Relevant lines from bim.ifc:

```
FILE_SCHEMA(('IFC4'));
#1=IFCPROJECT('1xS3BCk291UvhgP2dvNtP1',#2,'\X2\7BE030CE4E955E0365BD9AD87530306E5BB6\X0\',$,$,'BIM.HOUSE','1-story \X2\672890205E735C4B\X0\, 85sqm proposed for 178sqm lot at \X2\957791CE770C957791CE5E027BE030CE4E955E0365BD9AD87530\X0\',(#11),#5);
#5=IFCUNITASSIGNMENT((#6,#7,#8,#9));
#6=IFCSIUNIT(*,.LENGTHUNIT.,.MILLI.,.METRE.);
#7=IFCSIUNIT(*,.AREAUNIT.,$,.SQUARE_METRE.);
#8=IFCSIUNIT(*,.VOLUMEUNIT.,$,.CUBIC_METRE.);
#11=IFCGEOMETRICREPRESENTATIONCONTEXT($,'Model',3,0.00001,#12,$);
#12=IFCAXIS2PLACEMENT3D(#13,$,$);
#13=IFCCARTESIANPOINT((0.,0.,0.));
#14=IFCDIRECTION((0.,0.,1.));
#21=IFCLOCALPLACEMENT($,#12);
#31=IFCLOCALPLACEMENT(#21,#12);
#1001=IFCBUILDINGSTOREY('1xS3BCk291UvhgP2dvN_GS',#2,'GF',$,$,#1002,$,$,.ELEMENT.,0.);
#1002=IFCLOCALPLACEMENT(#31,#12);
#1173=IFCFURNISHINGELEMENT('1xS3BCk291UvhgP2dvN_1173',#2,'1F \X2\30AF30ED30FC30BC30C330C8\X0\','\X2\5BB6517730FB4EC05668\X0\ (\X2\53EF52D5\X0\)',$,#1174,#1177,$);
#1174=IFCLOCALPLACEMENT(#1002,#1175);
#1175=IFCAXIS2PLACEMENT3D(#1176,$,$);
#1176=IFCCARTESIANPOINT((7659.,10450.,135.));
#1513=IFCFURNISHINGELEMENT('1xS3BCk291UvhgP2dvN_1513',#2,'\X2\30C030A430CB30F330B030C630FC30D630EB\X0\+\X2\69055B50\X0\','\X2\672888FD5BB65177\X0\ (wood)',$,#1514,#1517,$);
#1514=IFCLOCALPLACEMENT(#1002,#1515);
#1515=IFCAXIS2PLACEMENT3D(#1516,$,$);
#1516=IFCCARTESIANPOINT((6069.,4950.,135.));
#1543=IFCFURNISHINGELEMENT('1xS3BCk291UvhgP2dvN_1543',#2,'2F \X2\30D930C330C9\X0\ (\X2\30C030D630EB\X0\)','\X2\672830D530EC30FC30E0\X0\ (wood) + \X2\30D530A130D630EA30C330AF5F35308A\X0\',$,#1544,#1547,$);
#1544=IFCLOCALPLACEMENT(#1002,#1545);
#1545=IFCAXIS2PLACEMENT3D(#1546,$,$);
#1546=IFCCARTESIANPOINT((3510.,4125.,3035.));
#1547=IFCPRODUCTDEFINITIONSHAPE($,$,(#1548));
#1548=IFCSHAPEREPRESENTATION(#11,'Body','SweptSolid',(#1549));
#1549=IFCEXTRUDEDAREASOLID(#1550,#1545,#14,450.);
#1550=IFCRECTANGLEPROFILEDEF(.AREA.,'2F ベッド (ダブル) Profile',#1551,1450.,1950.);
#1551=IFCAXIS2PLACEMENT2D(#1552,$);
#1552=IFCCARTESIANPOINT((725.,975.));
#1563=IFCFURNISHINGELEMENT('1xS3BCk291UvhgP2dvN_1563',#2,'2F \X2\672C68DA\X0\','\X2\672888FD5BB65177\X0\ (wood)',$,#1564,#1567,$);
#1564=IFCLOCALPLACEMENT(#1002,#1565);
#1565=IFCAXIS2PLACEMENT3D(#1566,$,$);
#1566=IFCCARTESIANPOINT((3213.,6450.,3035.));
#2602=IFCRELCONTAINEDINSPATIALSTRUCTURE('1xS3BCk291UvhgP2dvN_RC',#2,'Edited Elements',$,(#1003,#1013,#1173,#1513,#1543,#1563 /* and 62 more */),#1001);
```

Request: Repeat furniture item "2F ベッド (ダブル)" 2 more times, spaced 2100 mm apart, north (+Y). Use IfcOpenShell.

```python
import numpy as np
import ifcopenshell
import ifcopenshell.api.geometry
import ifcopenshell.api.root
import ifcopenshell.util.element
import ifcopenshell.util.placement
import ifcopenshell.util.unit

model = ifcopenshell.open("bim.ifc")
unit_scale = ifcopenshell.util.unit.calculate_unit_scale(model)


def reuse_history(source, copy):
    """copy_class also copies each property set's owner history, people and application; keep the originals."""
    for rel in copy.IsDefinedBy:
        if rel.is_a("IfcRelDefinesByProperties") and (history := rel.RelatingPropertyDefinition.OwnerHistory):
            rel.RelatingPropertyDefinition.OwnerHistory = source.OwnerHistory
            ifcopenshell.util.element.remove_deep2(model, history)


source = model.by_id(1543)
base = ifcopenshell.util.placement.get_local_placement(source.ObjectPlacement)
step = np.array([0.0, 1.0, 0.0]) * 2.1 / unit_scale

for i in range(1, 3):
    copy = ifcopenshell.api.root.copy_class(model, product=source)
    copy.Representation = ifcopenshell.util.element.copy_deep(
        model, source.Representation, exclude=["IfcGeometricRepresentationContext", "IfcRepresentationMap"]
    )
    reuse_history(source, copy)
    matrix = base.copy()
    matrix[:3, 3] += i * step
    print("added at", matrix[:3, 3].round(3) + 0.0)
    ifcopenshell.api.geometry.edit_object_placement(model, product=copy, matrix=matrix, is_si=False)

model.write("bim-out.ifc")
```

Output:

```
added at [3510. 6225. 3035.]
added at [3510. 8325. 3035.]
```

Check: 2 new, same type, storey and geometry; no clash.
